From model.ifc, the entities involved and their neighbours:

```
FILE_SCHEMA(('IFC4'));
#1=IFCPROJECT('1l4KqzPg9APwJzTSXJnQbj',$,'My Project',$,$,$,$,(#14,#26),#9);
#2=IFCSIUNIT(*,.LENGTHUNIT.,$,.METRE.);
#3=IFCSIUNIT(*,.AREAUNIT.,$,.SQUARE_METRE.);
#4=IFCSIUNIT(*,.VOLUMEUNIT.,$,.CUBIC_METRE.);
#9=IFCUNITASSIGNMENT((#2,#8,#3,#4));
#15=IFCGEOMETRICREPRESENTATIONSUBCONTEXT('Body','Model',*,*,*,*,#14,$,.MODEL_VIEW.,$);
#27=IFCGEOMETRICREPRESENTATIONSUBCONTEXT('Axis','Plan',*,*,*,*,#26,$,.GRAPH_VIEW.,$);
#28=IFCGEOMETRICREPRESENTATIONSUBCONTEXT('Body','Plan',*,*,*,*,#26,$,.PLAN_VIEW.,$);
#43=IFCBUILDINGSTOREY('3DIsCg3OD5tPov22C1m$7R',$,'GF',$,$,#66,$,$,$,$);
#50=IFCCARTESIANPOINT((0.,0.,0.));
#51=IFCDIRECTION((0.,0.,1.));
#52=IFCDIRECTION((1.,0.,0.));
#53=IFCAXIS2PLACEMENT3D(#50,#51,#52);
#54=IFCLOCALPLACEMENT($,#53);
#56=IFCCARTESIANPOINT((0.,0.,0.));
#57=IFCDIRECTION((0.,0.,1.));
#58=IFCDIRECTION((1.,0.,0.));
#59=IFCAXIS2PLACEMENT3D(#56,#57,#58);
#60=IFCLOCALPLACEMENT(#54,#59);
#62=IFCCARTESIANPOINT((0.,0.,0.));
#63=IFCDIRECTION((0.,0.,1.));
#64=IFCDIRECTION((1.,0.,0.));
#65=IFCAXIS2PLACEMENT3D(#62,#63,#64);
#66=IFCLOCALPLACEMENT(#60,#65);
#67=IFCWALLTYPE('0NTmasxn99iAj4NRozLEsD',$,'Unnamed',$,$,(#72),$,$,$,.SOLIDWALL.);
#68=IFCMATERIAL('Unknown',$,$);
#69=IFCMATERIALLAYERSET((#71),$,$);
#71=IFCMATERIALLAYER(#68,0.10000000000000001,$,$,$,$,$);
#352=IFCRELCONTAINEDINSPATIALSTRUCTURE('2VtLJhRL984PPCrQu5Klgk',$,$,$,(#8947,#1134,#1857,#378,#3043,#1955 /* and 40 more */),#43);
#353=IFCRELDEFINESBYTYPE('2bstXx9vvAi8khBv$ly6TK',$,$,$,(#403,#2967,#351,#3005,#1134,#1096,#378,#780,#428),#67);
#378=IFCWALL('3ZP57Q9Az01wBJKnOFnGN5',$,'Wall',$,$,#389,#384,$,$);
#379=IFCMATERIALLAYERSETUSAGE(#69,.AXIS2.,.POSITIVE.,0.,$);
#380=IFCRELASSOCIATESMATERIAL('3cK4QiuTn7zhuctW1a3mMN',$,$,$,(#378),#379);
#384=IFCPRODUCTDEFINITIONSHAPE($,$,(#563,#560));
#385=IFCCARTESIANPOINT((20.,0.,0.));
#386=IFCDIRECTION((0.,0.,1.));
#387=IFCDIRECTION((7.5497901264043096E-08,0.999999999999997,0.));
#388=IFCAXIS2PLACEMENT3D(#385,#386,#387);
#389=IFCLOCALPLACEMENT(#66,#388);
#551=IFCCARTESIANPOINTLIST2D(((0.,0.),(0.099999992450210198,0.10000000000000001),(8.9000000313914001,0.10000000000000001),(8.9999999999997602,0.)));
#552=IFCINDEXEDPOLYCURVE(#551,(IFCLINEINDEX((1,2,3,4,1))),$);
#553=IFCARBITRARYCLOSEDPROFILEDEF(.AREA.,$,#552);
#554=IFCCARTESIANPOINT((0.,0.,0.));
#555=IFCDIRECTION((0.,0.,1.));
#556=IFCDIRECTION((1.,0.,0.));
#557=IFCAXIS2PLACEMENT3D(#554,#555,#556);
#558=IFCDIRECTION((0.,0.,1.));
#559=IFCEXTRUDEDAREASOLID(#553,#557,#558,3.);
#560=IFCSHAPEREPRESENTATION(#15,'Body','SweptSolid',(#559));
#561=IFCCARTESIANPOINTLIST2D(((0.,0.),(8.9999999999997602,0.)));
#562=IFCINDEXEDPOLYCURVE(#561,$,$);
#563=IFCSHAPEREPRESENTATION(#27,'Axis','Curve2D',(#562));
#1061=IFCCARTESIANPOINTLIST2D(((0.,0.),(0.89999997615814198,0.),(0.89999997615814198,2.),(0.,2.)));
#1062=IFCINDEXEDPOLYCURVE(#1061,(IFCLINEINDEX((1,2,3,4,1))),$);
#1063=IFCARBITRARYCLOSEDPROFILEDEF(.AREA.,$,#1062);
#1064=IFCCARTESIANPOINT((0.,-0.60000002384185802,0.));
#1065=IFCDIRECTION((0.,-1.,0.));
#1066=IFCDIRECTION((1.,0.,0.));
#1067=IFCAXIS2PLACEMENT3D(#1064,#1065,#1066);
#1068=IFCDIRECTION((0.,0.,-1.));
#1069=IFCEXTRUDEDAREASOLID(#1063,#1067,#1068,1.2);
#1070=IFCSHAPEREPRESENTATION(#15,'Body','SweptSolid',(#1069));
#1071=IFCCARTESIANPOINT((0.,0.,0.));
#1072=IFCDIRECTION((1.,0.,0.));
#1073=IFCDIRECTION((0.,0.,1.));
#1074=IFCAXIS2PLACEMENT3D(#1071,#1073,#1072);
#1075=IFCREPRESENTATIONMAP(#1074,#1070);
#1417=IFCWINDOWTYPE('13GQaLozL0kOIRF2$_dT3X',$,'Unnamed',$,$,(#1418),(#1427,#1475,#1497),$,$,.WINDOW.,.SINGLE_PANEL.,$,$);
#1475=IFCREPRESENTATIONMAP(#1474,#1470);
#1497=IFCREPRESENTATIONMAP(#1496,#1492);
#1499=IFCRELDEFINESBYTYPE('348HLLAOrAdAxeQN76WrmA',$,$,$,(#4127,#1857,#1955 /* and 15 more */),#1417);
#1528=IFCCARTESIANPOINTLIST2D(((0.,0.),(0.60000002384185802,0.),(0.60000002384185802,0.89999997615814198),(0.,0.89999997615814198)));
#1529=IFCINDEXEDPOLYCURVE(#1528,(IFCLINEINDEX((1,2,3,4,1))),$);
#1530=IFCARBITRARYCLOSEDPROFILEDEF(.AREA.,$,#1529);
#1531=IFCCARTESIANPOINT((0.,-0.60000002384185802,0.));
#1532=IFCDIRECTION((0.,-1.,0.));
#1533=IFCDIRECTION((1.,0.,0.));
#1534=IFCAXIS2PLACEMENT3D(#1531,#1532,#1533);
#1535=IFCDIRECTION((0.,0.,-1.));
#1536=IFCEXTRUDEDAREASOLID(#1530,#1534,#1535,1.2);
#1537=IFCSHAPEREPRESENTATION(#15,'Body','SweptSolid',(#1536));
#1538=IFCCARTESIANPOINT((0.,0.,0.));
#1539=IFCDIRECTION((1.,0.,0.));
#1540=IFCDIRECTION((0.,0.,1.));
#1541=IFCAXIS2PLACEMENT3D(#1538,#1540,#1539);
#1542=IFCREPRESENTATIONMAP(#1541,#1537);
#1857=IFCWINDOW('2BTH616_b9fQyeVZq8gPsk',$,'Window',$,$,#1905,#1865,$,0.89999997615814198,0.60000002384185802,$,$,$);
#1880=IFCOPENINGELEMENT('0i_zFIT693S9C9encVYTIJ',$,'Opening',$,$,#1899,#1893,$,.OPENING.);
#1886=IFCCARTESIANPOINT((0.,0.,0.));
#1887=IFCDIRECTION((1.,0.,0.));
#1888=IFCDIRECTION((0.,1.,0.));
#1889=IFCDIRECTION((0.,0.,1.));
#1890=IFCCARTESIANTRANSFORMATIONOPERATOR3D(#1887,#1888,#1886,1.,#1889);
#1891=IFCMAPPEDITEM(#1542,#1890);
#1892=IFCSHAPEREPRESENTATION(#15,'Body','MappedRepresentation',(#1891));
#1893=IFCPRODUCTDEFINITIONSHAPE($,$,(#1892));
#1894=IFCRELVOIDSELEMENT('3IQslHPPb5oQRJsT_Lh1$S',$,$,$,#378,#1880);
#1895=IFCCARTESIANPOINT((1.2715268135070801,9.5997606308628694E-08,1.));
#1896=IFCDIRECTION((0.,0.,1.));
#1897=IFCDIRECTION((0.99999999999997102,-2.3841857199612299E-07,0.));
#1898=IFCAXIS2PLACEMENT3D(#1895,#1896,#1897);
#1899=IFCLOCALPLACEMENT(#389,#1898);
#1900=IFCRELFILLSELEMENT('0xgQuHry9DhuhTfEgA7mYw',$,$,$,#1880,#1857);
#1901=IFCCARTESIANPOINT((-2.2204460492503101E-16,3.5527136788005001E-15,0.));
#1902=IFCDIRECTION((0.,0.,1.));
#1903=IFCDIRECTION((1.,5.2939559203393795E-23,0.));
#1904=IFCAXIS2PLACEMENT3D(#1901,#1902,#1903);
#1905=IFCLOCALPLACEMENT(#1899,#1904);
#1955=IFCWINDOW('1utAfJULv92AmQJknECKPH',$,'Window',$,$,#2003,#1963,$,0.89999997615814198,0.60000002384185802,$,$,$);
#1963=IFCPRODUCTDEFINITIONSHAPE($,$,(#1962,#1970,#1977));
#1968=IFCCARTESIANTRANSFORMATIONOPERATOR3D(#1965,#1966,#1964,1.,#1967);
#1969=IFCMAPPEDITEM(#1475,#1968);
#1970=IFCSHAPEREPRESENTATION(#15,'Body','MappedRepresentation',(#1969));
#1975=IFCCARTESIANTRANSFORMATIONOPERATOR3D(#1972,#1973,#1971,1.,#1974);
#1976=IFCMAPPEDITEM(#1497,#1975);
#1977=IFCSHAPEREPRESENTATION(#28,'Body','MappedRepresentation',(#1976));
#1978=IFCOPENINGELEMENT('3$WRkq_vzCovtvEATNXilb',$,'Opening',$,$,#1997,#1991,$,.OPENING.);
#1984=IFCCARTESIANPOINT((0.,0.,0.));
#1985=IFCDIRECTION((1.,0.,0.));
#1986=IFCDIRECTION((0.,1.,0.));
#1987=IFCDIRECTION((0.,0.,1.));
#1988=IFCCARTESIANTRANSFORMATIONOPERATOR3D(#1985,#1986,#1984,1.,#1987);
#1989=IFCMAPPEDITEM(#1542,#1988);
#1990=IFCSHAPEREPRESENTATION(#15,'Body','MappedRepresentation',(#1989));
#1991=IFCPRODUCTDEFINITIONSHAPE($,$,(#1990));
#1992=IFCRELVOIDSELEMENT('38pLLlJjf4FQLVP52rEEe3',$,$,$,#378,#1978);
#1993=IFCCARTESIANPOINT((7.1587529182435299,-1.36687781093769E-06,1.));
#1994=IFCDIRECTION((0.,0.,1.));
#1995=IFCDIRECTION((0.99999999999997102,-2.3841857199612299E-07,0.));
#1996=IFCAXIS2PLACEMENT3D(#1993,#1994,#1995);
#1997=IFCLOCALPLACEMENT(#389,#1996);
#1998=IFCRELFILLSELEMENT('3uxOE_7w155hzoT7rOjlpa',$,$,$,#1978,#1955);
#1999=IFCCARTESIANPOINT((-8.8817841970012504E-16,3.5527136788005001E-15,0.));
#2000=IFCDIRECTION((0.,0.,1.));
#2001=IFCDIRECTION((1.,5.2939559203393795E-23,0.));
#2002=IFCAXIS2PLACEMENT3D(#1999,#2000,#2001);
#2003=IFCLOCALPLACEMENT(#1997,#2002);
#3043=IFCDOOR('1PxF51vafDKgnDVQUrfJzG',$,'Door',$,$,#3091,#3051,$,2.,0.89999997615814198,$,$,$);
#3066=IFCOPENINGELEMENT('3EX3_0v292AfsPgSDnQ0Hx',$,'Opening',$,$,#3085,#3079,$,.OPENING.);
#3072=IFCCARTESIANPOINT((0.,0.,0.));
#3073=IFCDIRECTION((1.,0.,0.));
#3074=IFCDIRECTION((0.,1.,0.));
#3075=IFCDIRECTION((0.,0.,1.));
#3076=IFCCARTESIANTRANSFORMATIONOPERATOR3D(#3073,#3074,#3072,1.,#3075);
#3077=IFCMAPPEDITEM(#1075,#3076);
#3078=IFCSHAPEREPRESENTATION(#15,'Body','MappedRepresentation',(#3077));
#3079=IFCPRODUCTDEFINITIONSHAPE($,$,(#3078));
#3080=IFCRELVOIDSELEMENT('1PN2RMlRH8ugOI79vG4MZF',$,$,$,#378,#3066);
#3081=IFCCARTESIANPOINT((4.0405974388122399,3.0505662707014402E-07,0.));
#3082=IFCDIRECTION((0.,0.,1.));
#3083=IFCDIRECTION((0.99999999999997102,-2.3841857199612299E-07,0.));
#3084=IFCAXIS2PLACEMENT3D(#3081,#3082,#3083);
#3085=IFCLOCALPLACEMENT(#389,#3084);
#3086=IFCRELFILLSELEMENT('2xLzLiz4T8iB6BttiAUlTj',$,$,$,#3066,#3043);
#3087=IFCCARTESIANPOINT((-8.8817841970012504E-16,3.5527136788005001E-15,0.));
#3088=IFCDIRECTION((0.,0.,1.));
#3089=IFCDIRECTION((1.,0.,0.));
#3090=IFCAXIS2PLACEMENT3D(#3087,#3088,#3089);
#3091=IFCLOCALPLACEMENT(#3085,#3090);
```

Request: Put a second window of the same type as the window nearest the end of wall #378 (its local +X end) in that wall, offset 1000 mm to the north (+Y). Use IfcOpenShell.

```python
import ifcopenshell
import ifcopenshell.api.feature
import ifcopenshell.api.geometry
import ifcopenshell.api.root
import ifcopenshell.geom
import ifcopenshell.util.element
import ifcopenshell.util.placement
import ifcopenshell.util.shape

model = ifcopenshell.open("model.ifc")
settings = ifcopenshell.geom.settings()


def volume(element):
    """Net volume in cubic metres, openings subtracted."""
    shape = ifcopenshell.geom.create_shape(settings, element)
    return ifcopenshell.util.shape.get_volume(shape.geometry)


window = model.by_guid("1utAfJULv92AmQJknECKPH")
opening = window.FillsVoids[0].RelatingOpeningElement
wall = opening.VoidsElements[0].RelatingBuildingElement
before = volume(wall)
shift = ifcopenshell.util.placement.get_local_placement(wall.ObjectPlacement)[:3, 0] * 1.0

# copy_class copies the void relationship, type, container and properties, but no geometry.
new_opening = ifcopenshell.api.root.copy_class(model, product=opening)
new_opening.Representation = ifcopenshell.util.element.copy_deep(
    model, opening.Representation, exclude=["IfcGeometricRepresentationContext", "IfcRepresentationMap"]
)
new_window = ifcopenshell.api.root.copy_class(model, product=window)
new_window.Representation = ifcopenshell.util.element.copy_deep(
    model, window.Representation, exclude=["IfcGeometricRepresentationContext", "IfcRepresentationMap"]
)
ifcopenshell.api.feature.add_filling(model, opening=new_opening, element=new_window)

for old, new in ((opening, new_opening), (window, new_window)):
    matrix = ifcopenshell.util.placement.get_local_placement(old.ObjectPlacement)
    matrix[:3, 3] += shift
    ifcopenshell.api.geometry.edit_object_placement(model, product=new, matrix=matrix, is_si=False)

after = volume(wall)

print(f"wall volume {before:.3f} -> {after:.3f} m3")

model.write("model-out.ifc")
```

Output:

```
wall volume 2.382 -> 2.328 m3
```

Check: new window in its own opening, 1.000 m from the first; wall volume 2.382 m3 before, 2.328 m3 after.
